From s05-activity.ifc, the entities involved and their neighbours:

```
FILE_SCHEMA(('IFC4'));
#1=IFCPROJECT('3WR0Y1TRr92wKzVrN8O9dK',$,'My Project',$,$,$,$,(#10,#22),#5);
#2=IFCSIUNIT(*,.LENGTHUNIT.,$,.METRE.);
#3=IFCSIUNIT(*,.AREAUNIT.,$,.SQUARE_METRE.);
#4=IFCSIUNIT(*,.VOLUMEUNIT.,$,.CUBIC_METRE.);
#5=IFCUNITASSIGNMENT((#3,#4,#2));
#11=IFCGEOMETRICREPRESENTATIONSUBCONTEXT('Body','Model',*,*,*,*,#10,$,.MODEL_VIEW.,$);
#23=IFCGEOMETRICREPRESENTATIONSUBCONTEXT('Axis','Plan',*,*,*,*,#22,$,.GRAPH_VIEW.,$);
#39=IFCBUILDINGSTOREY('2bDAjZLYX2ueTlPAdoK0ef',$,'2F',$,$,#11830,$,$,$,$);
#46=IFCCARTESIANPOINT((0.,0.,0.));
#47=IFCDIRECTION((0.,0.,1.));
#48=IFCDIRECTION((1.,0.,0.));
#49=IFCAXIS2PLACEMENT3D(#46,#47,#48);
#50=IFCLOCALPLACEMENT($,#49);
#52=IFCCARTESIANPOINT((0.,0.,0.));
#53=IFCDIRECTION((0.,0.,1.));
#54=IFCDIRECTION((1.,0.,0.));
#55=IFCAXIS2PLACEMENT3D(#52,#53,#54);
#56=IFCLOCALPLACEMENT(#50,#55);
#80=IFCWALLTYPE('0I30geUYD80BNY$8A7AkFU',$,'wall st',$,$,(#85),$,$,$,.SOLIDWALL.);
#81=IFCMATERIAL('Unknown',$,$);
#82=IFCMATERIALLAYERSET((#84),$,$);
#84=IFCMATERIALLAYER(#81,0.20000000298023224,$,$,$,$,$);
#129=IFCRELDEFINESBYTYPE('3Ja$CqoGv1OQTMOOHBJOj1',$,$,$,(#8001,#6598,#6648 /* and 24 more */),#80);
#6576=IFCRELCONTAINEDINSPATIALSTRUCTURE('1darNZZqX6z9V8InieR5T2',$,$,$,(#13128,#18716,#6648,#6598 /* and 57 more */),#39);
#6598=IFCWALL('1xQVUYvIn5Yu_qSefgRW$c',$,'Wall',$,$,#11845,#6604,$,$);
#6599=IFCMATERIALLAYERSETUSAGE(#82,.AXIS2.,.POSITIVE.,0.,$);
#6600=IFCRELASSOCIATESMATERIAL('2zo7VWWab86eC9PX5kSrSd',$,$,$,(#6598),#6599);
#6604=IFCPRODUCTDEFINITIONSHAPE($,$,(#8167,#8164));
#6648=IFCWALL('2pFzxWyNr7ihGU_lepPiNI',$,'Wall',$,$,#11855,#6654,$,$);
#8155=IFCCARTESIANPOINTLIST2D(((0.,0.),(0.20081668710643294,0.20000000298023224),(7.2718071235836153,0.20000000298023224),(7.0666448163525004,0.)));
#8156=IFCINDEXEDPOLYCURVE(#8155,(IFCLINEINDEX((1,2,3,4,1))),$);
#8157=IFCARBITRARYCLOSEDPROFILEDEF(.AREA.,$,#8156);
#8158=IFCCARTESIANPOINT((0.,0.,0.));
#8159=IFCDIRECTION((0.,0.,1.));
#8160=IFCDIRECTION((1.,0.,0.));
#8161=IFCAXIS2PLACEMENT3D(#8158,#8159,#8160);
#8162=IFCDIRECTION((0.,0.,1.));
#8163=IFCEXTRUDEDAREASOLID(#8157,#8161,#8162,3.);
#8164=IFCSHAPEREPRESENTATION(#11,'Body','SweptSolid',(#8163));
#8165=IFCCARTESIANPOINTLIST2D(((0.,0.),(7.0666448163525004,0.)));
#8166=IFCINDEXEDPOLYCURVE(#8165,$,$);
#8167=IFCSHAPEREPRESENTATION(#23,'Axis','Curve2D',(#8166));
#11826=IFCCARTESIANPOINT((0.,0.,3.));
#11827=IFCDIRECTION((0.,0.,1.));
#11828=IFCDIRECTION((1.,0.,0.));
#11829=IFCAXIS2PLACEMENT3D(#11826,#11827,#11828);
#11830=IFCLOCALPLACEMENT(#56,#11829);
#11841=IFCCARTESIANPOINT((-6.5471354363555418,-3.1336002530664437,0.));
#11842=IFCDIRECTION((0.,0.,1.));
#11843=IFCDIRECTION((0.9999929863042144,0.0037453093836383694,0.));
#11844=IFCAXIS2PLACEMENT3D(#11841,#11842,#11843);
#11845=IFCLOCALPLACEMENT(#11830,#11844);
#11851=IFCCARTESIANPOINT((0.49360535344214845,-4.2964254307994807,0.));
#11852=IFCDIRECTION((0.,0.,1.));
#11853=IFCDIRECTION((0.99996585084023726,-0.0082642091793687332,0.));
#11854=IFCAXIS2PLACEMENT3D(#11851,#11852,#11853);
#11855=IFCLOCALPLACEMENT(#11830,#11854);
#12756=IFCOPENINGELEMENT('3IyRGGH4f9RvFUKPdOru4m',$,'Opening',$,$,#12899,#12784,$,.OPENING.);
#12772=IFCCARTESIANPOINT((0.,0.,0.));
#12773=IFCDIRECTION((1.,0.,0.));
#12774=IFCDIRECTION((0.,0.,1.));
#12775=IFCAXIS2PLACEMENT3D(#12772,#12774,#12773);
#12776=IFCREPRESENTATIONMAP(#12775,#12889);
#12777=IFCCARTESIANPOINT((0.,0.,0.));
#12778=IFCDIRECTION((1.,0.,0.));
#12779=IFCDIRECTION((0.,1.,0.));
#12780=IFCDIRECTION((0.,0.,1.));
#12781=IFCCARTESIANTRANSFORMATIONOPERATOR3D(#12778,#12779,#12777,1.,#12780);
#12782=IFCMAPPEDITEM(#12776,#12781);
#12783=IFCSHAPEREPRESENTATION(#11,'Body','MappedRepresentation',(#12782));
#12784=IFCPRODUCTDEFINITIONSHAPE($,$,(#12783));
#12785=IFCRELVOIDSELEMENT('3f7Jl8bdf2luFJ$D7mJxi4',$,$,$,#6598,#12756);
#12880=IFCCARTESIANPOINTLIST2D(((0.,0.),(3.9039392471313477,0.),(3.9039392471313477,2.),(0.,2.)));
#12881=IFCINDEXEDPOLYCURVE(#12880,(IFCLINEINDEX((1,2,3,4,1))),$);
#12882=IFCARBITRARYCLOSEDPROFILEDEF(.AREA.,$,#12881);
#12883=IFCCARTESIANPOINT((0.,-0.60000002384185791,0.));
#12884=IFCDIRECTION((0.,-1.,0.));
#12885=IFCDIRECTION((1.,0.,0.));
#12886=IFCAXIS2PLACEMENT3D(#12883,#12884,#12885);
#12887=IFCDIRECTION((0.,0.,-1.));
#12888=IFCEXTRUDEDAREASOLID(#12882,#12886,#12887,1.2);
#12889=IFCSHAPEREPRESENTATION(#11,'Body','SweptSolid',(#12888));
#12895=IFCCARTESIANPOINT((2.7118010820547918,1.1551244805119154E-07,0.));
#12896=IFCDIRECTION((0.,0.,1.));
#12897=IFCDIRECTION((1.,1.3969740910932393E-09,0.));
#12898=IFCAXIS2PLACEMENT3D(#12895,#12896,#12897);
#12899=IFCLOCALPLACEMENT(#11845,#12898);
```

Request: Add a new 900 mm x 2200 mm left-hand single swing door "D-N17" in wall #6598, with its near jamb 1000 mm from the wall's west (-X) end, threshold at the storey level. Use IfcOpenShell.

```python
import numpy as np
import ifcopenshell
import ifcopenshell.api.feature
import ifcopenshell.api.geometry
import ifcopenshell.api.root
import ifcopenshell.api.spatial
import ifcopenshell.geom
import ifcopenshell.util.element
import ifcopenshell.util.placement
import ifcopenshell.util.representation
import ifcopenshell.util.shape
import ifcopenshell.util.unit

model = ifcopenshell.open("s05-activity.ifc")
unit_scale = ifcopenshell.util.unit.calculate_unit_scale(model)
settings = ifcopenshell.geom.settings()


def volume(element):
    """Net volume in cubic metres, openings subtracted."""
    shape = ifcopenshell.geom.create_shape(settings, element)
    return ifcopenshell.util.shape.get_volume(shape.geometry)


wall = model.by_guid("1xQVUYvIn5Yu_qSefgRW$c")
storey = ifcopenshell.util.element.get_container(wall, ifc_class="IfcBuildingStorey")
context = ifcopenshell.util.representation.get_context(model, "Model", "Body", "MODEL_VIEW")
before = volume(wall)

width, height, from_end, sill = 0.9, 2.2, 1, 0.0  # metres

# The wall runs along its own X axis, and the end named is its -X end.
wall_shape = ifcopenshell.geom.create_shape(settings, wall)
x, y, z = ifcopenshell.util.shape.get_vertices(wall_shape.geometry).T
start = x.min() + from_end
face, thickness = float(y.min()), float(y.max() - y.min())
wall_matrix = ifcopenshell.util.placement.get_local_placement(wall.ObjectPlacement)
level = ifcopenshell.util.placement.get_local_placement(storey.ObjectPlacement)[2, 3]


def in_wall(x, y):
    """Placement at x, y metres in the wall's axes, at sill height."""
    matrix = wall_matrix.copy()
    matrix[:, 3] = wall_matrix @ np.array([x / unit_scale, y / unit_scale, 0.0, 1.0])
    matrix[2, 3] = level + sill / unit_scale
    return matrix


# Opening: a box that overshoots both wall faces by 50 mm.
opening = ifcopenshell.api.root.create_entity(model, ifc_class="IfcOpeningElement", predefined_type="OPENING")
box = ifcopenshell.api.geometry.add_wall_representation(
    model, context=context, length=width, height=height, thickness=thickness + 0.1
)
ifcopenshell.api.geometry.assign_representation(model, product=opening, representation=box)
ifcopenshell.api.geometry.edit_object_placement(model, product=opening, matrix=in_wall(start, face - 0.05), is_si=False)
ifcopenshell.api.feature.add_feature(model, feature=opening, element=wall)

door = ifcopenshell.api.root.create_entity(model, ifc_class="IfcDoor", name="D-N17", predefined_type="DOOR")
door.OverallWidth, door.OverallHeight = width / unit_scale, height / unit_scale
door.OperationType = "SINGLE_SWING_LEFT"
body = ifcopenshell.api.geometry.add_door_representation(
    model,
    context=context,
    overall_width=door.OverallWidth,
    overall_height=door.OverallHeight,
    operation_type="SINGLE_SWING_LEFT",
    lining_properties={"LiningDepth": thickness / unit_scale, "ThresholdDepth": thickness / unit_scale},
)
ifcopenshell.api.geometry.assign_representation(model, product=door, representation=body)
ifcopenshell.api.spatial.assign_container(model, products=[door], relating_structure=storey)
ifcopenshell.api.feature.add_filling(model, opening=opening, element=door)

# The lining spans the wall, so the door starts at the wall face.
ifcopenshell.api.geometry.edit_object_placement(model, product=door, matrix=in_wall(start, face), is_si=False)

after = volume(wall)

print(f"wall volume {before:.3f} -> {after:.3f} m3")

model.write("s05-activity_rev.ifc")
```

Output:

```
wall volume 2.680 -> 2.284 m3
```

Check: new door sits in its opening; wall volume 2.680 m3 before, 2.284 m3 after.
